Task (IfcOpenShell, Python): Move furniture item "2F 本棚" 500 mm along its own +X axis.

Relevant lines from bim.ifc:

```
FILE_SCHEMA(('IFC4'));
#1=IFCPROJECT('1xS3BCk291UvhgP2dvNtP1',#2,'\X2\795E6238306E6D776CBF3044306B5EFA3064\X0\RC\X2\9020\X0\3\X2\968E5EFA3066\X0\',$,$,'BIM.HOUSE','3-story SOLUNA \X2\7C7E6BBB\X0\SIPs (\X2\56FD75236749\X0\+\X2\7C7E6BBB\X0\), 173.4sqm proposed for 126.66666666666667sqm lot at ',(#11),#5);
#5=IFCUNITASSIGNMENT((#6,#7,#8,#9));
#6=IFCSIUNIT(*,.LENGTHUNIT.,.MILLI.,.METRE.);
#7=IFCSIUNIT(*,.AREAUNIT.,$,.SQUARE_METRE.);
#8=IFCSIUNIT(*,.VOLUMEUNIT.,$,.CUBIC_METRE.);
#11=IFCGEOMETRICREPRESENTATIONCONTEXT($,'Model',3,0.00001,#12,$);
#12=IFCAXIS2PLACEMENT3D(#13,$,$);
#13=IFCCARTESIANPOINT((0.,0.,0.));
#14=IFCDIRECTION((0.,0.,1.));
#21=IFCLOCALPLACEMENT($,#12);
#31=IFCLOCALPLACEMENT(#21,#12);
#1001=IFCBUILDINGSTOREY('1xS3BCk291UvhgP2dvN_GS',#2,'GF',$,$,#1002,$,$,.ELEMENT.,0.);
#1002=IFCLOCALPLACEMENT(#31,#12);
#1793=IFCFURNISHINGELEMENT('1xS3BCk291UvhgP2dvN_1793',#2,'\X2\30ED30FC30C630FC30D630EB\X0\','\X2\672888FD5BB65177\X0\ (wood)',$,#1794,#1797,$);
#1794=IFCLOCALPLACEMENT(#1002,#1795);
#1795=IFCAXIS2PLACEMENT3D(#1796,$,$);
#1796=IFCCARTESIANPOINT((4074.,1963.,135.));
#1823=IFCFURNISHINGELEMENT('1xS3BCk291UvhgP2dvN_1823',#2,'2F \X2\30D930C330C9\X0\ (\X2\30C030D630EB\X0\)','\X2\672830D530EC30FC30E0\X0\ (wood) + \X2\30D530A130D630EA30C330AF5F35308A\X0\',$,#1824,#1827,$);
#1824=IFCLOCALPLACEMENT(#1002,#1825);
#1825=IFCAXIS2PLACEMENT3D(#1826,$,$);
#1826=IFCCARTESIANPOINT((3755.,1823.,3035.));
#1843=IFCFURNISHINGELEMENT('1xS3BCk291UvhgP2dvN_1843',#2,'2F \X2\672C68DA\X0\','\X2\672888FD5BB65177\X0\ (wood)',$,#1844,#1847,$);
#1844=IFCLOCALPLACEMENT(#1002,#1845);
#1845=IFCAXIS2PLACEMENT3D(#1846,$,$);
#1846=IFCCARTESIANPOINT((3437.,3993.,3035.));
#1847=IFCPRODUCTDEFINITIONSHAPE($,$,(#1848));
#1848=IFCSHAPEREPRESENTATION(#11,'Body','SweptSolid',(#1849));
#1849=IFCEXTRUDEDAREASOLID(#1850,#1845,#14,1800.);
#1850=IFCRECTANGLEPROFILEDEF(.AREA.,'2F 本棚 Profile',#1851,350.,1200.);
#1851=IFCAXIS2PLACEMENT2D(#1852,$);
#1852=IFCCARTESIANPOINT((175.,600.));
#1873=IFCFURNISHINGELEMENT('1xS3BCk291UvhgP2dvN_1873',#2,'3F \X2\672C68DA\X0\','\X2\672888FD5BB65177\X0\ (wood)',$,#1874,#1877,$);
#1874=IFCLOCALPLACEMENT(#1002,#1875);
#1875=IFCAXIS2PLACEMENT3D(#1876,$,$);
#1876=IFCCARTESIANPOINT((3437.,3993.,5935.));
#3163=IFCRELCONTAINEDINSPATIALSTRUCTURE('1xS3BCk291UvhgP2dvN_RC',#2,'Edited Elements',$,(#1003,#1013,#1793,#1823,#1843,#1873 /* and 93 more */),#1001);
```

```python
import ifcopenshell
import ifcopenshell.api.geometry
import ifcopenshell.util.placement

model = ifcopenshell.open("bim.ifc")

item = model.by_guid("1xS3BCk291UvhgP2dvN_1843")
matrix = ifcopenshell.util.placement.get_local_placement(item.ObjectPlacement)
matrix[:3, 3] += matrix[:3, 0] * 500.0
ifcopenshell.api.geometry.edit_object_placement(model, product=item, matrix=matrix, is_si=False)

print(ifcopenshell.util.placement.get_local_placement(item.ObjectPlacement).round(3) + 0.0)

model.write("bim_updated.ifc")
```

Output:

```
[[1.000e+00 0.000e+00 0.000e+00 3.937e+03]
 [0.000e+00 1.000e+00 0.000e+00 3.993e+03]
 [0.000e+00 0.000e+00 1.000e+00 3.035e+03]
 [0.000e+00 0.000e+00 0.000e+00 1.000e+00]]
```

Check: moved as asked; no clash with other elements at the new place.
